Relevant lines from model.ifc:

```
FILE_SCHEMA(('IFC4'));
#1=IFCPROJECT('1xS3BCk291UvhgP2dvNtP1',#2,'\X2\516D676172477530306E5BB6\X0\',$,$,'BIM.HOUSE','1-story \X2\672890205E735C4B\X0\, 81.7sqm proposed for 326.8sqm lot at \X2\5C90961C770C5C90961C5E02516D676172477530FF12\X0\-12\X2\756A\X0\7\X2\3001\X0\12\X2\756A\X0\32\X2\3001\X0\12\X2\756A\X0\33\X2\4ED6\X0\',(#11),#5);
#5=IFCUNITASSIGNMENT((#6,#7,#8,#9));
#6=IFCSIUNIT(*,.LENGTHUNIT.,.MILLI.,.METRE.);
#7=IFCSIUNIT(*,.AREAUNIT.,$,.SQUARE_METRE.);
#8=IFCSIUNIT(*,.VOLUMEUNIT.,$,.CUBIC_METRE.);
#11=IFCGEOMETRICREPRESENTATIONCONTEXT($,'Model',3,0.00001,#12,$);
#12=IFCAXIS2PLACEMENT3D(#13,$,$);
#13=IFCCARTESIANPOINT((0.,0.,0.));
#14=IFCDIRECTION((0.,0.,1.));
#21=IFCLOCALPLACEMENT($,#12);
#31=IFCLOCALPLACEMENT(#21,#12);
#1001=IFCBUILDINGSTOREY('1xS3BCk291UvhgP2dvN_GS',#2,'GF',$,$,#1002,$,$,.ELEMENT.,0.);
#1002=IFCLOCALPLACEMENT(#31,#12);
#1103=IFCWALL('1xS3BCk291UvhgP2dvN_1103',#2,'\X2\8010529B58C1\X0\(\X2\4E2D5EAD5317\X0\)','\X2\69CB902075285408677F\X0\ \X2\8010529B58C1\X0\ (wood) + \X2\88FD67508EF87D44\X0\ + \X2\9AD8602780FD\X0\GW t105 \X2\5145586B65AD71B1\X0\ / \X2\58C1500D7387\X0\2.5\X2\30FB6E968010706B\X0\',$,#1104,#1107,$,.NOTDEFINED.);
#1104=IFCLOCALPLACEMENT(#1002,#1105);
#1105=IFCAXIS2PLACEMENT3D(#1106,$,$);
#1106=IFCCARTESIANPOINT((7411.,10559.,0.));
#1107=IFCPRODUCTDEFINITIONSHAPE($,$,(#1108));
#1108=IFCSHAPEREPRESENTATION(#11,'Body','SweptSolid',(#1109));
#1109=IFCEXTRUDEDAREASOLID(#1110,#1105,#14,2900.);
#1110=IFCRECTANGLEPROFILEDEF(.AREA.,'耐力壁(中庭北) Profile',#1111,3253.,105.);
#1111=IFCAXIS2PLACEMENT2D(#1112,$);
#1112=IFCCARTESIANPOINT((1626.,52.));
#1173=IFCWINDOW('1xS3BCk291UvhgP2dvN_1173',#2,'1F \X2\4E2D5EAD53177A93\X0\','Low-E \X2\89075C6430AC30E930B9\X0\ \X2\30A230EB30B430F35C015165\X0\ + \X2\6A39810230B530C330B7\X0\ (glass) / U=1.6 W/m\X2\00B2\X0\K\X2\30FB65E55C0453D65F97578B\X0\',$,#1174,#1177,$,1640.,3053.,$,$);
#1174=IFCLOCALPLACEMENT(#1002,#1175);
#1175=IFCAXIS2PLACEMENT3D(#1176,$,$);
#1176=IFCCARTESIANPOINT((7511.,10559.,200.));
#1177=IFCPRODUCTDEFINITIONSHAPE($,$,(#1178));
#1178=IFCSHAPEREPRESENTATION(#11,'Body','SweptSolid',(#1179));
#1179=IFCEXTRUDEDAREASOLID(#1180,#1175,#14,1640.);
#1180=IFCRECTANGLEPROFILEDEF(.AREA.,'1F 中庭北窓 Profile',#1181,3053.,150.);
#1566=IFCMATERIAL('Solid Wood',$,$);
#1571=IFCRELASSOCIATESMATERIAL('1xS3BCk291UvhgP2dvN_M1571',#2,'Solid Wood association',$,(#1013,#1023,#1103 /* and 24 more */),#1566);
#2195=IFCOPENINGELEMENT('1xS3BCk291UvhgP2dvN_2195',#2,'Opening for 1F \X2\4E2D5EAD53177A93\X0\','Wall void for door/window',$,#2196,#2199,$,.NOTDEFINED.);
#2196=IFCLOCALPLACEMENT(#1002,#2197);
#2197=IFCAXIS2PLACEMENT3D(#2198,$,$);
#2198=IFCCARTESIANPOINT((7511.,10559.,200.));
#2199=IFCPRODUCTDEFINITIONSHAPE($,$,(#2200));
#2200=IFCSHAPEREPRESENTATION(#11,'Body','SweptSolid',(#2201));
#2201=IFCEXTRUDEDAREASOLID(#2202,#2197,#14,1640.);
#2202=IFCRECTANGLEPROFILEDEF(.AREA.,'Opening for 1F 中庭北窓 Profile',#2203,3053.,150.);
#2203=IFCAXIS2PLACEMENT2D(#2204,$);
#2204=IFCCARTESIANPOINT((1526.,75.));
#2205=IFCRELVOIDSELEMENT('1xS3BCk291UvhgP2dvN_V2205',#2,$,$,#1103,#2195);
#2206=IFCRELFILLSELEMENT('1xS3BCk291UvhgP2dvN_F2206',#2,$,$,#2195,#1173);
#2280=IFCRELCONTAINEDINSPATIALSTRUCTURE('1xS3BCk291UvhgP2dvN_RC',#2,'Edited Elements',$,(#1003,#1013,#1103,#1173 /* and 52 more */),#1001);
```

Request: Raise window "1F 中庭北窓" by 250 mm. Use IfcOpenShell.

```python
import numpy as np
import ifcopenshell
import ifcopenshell.api.geometry
import ifcopenshell.util.placement
import ifcopenshell.util.unit

model = ifcopenshell.open("model.ifc")
unit_scale = ifcopenshell.util.unit.calculate_unit_scale(model)

window = model.by_guid("1xS3BCk291UvhgP2dvN_1173")
opening = window.FillsVoids[0].RelatingOpeningElement
dz = 0.25 / unit_scale

shift = np.array([0.0, 0.0, dz])
# The window is not placed relative to its opening, so move both.
for product in (opening, window):
    matrix = ifcopenshell.util.placement.get_local_placement(product.ObjectPlacement)
    matrix[:3, 3] += shift
    ifcopenshell.api.geometry.edit_object_placement(model, product=product, matrix=matrix, is_si=False)

print(f"moved by {dz * unit_scale:+.3f} m")

model.write("model_updated.ifc")
```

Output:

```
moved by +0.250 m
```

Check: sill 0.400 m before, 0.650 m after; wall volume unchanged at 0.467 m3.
